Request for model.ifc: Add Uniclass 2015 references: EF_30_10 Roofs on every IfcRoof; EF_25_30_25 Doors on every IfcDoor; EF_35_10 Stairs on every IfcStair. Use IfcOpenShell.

First a look at what the model holds.

```python
import ifcopenshell

model = ifcopenshell.open("model.ifc")
print(model.schema)
print("classifications:", [c.Name for c in model.by_type("IfcClassification")])
for ifc_class in ("IfcDoor", "IfcRoof", "IfcStair", "IfcWall", "IfcWindow"):
    print(ifc_class, len(model.by_type(ifc_class)))
```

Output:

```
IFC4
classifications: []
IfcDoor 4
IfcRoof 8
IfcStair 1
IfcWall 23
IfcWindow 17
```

```python
import ifcopenshell
import ifcopenshell.api.classification

model = ifcopenshell.open("model.ifc")

system = ifcopenshell.api.classification.add_classification(model, classification="Uniclass 2015")

codes = {
    "IfcRoof": ("EF_30_10", "Roofs"),
    "IfcDoor": ("EF_25_30_25", "Doors"),
    "IfcStair": ("EF_35_10", "Stairs"),
}
for ifc_class, (code, name) in codes.items():
    products = model.by_type(ifc_class)
    ifcopenshell.api.classification.add_reference(
        model, products=products, classification=system, identification=code, name=name
    )
    print(code, len(products))

model.write("model-out.ifc")
```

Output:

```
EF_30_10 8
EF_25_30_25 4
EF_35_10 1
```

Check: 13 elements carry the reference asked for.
